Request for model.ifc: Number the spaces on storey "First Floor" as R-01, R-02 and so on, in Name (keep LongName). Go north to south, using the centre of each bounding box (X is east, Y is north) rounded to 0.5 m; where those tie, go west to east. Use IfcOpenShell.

First a look at what the model holds.

```python
import ifcopenshell
import ifcopenshell.util.element
import ifcopenshell.util.placement

model = ifcopenshell.open("model.ifc")
print(model.schema)
storey = next(s for s in model.by_type("IfcBuildingStorey") if s.Name == "First Floor")
spaces = [e for e in ifcopenshell.util.element.get_decomposition(storey) if e.is_a("IfcSpace")]
for e in sorted(spaces, key=lambda e: e.id()):
    origin = ifcopenshell.util.placement.get_local_placement(e.ObjectPlacement)[:3, 3]
    print(e.id(), e.Name, e.LongName, origin.round(2) + 0.0, sep=" | ")
```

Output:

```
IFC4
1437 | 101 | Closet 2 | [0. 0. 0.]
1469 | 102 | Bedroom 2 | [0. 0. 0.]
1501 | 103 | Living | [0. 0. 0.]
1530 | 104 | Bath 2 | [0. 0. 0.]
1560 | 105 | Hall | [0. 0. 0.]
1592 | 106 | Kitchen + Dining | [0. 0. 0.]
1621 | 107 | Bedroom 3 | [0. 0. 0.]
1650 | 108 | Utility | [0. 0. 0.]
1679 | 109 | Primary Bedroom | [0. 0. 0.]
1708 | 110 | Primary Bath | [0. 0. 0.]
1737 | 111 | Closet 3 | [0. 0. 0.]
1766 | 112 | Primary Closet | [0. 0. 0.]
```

```python
import ifcopenshell
import ifcopenshell.geom
import ifcopenshell.util.element
import ifcopenshell.util.shape

model = ifcopenshell.open("model.ifc")
settings = ifcopenshell.geom.settings()
settings.set("use-world-coords", True)


def centre(element):
    shape = ifcopenshell.geom.create_shape(settings, element)
    return ifcopenshell.util.shape.get_bbox_centroid(shape.geometry)


storey = next(s for s in model.by_type("IfcBuildingStorey") if s.Name == "First Floor")
spaces = [e for e in ifcopenshell.util.element.get_decomposition(storey) if e.is_a("IfcSpace")]

# Insertion points can sit at a corner or the storey origin, so sort by the geometry (in metres).
centres = {e: centre(e) for e in spaces}
spaces.sort(key=lambda e: (-round(centres[e][1] / 0.5), centres[e][0]))

for i, e in enumerate(spaces, start=1):
    number = f"R-{i:02d}"
    e.Name = number
    print(e.id(), number)

model.write("model_updated.ifc")
```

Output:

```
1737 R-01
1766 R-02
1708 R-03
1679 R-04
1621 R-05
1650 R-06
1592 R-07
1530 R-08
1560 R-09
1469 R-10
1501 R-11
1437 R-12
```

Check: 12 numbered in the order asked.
